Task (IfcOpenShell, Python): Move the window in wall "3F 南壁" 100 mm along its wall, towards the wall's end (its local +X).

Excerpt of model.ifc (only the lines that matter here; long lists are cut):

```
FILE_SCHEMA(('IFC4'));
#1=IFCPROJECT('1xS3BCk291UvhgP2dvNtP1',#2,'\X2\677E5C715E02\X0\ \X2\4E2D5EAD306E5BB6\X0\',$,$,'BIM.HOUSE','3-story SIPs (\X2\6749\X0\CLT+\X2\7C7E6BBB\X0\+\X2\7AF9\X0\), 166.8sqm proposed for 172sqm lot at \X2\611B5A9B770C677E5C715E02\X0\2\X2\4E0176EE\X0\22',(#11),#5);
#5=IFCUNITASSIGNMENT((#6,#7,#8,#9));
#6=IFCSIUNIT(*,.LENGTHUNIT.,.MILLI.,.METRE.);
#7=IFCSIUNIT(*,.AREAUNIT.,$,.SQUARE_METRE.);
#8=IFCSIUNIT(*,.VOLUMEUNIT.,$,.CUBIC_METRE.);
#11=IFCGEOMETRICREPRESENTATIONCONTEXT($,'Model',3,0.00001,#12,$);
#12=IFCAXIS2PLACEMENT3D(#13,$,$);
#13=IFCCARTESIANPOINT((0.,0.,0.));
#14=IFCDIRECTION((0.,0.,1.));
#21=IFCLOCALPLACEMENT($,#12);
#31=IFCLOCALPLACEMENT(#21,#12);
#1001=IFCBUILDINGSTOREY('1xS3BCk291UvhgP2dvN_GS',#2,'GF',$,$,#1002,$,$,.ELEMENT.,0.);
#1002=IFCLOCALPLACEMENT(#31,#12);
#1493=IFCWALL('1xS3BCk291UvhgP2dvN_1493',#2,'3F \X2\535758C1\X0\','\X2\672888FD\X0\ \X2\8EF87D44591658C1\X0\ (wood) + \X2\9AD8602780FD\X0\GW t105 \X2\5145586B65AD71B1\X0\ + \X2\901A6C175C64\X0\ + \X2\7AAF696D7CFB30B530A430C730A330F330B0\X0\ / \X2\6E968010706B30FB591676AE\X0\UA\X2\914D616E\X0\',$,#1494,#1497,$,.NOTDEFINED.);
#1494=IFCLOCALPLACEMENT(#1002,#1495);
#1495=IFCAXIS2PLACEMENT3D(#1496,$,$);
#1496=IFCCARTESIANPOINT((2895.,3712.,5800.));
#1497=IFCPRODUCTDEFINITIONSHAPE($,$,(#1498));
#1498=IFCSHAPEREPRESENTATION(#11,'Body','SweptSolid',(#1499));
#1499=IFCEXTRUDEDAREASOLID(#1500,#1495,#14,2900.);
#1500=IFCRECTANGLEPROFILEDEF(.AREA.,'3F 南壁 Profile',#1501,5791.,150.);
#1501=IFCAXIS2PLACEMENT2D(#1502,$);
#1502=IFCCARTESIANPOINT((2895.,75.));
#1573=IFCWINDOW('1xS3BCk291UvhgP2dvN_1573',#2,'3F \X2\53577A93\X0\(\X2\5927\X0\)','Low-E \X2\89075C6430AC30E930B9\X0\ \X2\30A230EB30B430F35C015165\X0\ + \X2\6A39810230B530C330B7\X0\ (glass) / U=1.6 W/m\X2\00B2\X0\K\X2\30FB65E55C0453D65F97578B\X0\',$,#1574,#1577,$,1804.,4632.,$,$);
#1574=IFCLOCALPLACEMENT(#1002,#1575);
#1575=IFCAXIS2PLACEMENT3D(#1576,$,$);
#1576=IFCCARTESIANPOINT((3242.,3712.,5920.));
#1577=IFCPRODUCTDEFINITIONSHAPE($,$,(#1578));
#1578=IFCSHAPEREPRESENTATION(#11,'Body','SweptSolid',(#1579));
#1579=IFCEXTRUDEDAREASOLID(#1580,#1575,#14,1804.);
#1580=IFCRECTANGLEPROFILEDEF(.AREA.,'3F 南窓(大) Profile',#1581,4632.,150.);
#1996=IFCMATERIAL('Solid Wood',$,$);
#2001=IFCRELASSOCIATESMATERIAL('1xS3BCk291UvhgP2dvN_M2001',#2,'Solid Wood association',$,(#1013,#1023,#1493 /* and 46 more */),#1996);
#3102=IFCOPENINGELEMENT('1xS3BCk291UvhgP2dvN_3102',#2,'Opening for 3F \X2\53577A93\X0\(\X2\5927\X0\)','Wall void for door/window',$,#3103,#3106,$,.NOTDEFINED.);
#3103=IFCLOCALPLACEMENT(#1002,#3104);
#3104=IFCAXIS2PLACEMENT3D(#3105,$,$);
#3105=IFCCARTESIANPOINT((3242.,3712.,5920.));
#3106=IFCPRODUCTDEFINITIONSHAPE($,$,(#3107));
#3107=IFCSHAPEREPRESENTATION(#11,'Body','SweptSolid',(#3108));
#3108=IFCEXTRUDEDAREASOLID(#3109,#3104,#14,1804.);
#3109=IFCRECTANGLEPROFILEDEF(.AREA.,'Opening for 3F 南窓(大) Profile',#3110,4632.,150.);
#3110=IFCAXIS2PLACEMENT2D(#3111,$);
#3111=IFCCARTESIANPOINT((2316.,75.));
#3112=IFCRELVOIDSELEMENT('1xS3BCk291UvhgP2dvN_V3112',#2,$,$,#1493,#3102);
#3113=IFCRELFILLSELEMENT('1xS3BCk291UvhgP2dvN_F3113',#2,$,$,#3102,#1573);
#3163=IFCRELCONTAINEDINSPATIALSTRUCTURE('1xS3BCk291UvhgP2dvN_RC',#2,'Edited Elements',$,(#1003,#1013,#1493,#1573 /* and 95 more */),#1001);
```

```python
import ifcopenshell
import ifcopenshell.api.geometry
import ifcopenshell.util.placement

model = ifcopenshell.open("model.ifc")

window = model.by_guid("1xS3BCk291UvhgP2dvN_1573")
opening = window.FillsVoids[0].RelatingOpeningElement
wall = opening.VoidsElements[0].RelatingBuildingElement

wall_matrix = ifcopenshell.util.placement.get_local_placement(wall.ObjectPlacement)
shift = wall_matrix[:3, 0] * 100.0
before = ifcopenshell.util.placement.get_local_placement(window.ObjectPlacement)[:3, 3].copy()

# The window is not placed relative to its opening, so move both.
for product in (opening, window):
    matrix = ifcopenshell.util.placement.get_local_placement(product.ObjectPlacement)
    matrix[:3, 3] += shift
    ifcopenshell.api.geometry.edit_object_placement(model, product=product, matrix=matrix, is_si=False)

after = ifcopenshell.util.placement.get_local_placement(window.ObjectPlacement)[:3, 3]
print("window moved by", (after - before).round(3) + 0.0)

model.write("model-out.ifc")
```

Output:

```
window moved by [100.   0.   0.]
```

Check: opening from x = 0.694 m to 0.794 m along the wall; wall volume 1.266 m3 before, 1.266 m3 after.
